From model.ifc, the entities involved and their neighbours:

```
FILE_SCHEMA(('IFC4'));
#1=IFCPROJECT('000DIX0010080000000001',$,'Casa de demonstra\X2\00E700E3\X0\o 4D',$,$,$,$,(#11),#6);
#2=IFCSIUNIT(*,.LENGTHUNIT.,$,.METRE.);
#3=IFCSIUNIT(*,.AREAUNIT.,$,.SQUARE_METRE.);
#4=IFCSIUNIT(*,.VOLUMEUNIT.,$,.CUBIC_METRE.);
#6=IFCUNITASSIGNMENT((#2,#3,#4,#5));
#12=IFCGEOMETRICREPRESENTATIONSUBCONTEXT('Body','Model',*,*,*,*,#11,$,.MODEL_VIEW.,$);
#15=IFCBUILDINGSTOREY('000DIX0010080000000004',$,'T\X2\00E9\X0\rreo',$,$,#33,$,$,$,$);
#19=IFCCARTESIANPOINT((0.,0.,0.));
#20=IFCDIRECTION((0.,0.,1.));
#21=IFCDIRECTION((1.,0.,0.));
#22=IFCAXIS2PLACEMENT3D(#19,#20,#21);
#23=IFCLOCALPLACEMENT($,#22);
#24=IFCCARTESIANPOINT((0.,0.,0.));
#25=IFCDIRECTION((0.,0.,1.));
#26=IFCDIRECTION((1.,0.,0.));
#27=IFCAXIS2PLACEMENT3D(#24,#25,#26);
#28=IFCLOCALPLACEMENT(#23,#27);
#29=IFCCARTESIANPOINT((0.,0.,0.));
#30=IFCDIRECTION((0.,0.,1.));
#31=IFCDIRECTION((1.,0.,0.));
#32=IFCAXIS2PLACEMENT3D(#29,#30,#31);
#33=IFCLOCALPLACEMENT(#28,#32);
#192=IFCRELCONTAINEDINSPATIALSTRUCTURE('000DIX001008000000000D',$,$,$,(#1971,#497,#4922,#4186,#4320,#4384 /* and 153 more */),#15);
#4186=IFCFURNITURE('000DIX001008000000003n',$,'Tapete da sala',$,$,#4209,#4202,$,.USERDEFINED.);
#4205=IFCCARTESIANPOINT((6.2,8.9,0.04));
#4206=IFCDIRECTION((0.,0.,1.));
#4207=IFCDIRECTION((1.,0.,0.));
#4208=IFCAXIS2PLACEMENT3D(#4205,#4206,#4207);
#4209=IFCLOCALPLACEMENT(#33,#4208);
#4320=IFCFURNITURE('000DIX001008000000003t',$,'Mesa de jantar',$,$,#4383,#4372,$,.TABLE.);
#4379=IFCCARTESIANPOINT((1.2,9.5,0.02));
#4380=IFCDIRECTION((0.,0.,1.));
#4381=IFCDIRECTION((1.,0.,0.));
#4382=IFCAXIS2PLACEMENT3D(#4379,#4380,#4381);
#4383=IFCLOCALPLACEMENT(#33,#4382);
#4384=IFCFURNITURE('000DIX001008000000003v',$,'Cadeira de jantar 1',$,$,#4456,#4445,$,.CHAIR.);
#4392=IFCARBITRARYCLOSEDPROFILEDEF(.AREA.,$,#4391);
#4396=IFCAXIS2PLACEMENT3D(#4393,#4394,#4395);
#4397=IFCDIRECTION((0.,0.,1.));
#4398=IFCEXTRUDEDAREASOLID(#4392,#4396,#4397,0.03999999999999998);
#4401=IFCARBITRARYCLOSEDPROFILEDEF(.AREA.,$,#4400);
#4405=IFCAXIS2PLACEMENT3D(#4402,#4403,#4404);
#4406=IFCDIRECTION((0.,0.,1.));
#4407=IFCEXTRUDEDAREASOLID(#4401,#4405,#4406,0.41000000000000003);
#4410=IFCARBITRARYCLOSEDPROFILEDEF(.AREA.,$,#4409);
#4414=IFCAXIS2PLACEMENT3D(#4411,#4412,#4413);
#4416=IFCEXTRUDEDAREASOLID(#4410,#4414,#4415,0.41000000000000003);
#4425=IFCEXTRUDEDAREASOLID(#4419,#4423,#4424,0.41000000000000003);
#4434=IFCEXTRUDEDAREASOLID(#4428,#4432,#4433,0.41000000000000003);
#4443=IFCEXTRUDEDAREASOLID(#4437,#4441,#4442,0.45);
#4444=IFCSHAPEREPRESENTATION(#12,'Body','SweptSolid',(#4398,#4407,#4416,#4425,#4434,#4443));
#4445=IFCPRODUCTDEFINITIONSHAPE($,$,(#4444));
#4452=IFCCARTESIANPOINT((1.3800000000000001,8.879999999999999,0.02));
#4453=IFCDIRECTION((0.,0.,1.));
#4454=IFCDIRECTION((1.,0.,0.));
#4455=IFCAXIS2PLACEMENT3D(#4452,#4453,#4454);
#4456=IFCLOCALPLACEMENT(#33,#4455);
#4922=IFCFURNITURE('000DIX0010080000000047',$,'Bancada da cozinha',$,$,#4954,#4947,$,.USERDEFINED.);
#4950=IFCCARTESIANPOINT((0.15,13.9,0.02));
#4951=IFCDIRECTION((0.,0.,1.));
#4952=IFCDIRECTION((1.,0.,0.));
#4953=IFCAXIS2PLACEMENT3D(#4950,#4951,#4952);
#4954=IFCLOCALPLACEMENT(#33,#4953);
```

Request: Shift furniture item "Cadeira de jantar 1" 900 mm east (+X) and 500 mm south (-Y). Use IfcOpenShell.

```python
import ifcopenshell
import ifcopenshell.api.geometry
import ifcopenshell.util.placement
import ifcopenshell.util.unit

model = ifcopenshell.open("model.ifc")
unit_scale = ifcopenshell.util.unit.calculate_unit_scale(model)

item = model.by_guid("000DIX001008000000003v")
matrix = ifcopenshell.util.placement.get_local_placement(item.ObjectPlacement)
matrix[0, 3] += 0.9 / unit_scale
matrix[1, 3] -= 0.5 / unit_scale
ifcopenshell.api.geometry.edit_object_placement(model, product=item, matrix=matrix, is_si=False)

print(ifcopenshell.util.placement.get_local_placement(item.ObjectPlacement).round(3) + 0.0)

model.write("model_v2.ifc")
```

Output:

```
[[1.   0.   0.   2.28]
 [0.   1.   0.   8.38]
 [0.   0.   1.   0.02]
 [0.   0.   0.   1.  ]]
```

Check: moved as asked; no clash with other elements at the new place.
